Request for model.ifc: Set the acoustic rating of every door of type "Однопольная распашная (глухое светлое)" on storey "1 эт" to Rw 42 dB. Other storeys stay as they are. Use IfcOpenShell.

First a look at what the model holds.

```python
import ifcopenshell
import ifcopenshell.util.element

model = ifcopenshell.open("model.ifc")
print(model.schema)
storey = next(s for s in model.by_type("IfcBuildingStorey") if s.Name == "1 эт")
doors = [e for e in ifcopenshell.util.element.get_decomposition(storey) if e.is_a("IfcDoor")]
seen = {}
for e in doors:
    element_type = ifcopenshell.util.element.get_type(e)
    key = (element_type.Name if element_type != e and element_type else None, ifcopenshell.util.element.get_pset(e, "Pset_DoorCommon", "AcousticRating"))
    seen[key] = seen.get(key, 0) + 1
for (name, value), count in sorted(seen.items(), key=str):
    print(count, "x", name, "|", value)
```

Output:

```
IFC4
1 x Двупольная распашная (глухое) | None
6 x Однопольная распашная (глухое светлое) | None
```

```python
import ifcopenshell
import ifcopenshell.api.pset
import ifcopenshell.util.element

model = ifcopenshell.open("model.ifc")

storey = next(s for s in model.by_type("IfcBuildingStorey") if s.Name == "1 эт")
doors = [e for e in ifcopenshell.util.element.get_decomposition(storey) if e.is_a("IfcDoor")]

count = 0
for e in doors:
    element_type = ifcopenshell.util.element.get_type(e)
    if element_type in (None, e) or element_type.Name != "Однопольная распашная (глухое светлое)":
        continue
    # add_pset returns the element's existing set when there is one.
    pset = ifcopenshell.api.pset.add_pset(model, product=e, name="Pset_DoorCommon")
    ifcopenshell.api.pset.edit_pset(model, pset=pset, properties={"AcousticRating": "Rw 42 dB"})
    count += 1

print(count, "doors updated")

model.write("model_v2.ifc")
```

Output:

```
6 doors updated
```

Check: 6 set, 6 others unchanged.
